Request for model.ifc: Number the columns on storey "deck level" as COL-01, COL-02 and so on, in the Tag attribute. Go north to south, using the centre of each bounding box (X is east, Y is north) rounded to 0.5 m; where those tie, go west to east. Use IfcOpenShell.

First a look at what the model holds.

```python
import ifcopenshell
import ifcopenshell.util.element
import ifcopenshell.util.placement

model = ifcopenshell.open("model.ifc")
print(model.schema)
storey = next(s for s in model.by_type("IfcBuildingStorey") if s.Name == "deck level")
columns = [e for e in ifcopenshell.util.element.get_decomposition(storey) if e.is_a("IfcColumn")]
for e in sorted(columns, key=lambda e: e.id()):
    origin = ifcopenshell.util.placement.get_local_placement(e.ObjectPlacement)[:3, 3]
    print(e.id(), e.Tag, e.Name, origin.round(2) + 0.0, sep=" | ")
```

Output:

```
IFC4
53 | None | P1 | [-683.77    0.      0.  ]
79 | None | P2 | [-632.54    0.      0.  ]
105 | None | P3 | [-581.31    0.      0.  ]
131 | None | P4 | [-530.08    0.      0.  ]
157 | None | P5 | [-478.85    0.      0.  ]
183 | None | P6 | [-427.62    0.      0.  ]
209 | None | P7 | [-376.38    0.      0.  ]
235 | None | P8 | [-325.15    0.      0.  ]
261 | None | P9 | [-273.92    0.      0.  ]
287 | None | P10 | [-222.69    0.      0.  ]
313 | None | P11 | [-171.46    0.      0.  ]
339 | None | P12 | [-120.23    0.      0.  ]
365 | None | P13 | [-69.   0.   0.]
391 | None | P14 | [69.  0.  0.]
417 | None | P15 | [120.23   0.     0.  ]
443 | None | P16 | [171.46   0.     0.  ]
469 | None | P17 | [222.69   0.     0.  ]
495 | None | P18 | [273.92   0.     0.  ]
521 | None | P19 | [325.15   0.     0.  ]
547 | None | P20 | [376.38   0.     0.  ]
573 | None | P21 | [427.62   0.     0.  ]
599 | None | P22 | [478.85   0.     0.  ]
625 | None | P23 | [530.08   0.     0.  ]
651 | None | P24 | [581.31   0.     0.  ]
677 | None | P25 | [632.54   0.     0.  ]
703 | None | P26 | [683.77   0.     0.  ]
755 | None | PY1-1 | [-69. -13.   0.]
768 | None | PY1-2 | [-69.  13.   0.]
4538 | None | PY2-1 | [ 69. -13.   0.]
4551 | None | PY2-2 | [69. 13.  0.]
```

```python
import ifcopenshell
import ifcopenshell.geom
import ifcopenshell.util.element
import ifcopenshell.util.shape

model = ifcopenshell.open("model.ifc")
settings = ifcopenshell.geom.settings()
settings.set("use-world-coords", True)


def centre(element):
    shape = ifcopenshell.geom.create_shape(settings, element)
    return ifcopenshell.util.shape.get_bbox_centroid(shape.geometry)


storey = next(s for s in model.by_type("IfcBuildingStorey") if s.Name == "deck level")
columns = [e for e in ifcopenshell.util.element.get_decomposition(storey) if e.is_a("IfcColumn")]

# Insertion points can sit at a corner or the storey origin, so sort by the geometry (in metres).
centres = {e: centre(e) for e in columns}
columns.sort(key=lambda e: (-round(centres[e][1] / 0.5), centres[e][0]))

for i, e in enumerate(columns, start=1):
    number = f"COL-{i:02d}"
    e.Tag = number
    print(e.id(), number)

model.write("model-out.ifc")
```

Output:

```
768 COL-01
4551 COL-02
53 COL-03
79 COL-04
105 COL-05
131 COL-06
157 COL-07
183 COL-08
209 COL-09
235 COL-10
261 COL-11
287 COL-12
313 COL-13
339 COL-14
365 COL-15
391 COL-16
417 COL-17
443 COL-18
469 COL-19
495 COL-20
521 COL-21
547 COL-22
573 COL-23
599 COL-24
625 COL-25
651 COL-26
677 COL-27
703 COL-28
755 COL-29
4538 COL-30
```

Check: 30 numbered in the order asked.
